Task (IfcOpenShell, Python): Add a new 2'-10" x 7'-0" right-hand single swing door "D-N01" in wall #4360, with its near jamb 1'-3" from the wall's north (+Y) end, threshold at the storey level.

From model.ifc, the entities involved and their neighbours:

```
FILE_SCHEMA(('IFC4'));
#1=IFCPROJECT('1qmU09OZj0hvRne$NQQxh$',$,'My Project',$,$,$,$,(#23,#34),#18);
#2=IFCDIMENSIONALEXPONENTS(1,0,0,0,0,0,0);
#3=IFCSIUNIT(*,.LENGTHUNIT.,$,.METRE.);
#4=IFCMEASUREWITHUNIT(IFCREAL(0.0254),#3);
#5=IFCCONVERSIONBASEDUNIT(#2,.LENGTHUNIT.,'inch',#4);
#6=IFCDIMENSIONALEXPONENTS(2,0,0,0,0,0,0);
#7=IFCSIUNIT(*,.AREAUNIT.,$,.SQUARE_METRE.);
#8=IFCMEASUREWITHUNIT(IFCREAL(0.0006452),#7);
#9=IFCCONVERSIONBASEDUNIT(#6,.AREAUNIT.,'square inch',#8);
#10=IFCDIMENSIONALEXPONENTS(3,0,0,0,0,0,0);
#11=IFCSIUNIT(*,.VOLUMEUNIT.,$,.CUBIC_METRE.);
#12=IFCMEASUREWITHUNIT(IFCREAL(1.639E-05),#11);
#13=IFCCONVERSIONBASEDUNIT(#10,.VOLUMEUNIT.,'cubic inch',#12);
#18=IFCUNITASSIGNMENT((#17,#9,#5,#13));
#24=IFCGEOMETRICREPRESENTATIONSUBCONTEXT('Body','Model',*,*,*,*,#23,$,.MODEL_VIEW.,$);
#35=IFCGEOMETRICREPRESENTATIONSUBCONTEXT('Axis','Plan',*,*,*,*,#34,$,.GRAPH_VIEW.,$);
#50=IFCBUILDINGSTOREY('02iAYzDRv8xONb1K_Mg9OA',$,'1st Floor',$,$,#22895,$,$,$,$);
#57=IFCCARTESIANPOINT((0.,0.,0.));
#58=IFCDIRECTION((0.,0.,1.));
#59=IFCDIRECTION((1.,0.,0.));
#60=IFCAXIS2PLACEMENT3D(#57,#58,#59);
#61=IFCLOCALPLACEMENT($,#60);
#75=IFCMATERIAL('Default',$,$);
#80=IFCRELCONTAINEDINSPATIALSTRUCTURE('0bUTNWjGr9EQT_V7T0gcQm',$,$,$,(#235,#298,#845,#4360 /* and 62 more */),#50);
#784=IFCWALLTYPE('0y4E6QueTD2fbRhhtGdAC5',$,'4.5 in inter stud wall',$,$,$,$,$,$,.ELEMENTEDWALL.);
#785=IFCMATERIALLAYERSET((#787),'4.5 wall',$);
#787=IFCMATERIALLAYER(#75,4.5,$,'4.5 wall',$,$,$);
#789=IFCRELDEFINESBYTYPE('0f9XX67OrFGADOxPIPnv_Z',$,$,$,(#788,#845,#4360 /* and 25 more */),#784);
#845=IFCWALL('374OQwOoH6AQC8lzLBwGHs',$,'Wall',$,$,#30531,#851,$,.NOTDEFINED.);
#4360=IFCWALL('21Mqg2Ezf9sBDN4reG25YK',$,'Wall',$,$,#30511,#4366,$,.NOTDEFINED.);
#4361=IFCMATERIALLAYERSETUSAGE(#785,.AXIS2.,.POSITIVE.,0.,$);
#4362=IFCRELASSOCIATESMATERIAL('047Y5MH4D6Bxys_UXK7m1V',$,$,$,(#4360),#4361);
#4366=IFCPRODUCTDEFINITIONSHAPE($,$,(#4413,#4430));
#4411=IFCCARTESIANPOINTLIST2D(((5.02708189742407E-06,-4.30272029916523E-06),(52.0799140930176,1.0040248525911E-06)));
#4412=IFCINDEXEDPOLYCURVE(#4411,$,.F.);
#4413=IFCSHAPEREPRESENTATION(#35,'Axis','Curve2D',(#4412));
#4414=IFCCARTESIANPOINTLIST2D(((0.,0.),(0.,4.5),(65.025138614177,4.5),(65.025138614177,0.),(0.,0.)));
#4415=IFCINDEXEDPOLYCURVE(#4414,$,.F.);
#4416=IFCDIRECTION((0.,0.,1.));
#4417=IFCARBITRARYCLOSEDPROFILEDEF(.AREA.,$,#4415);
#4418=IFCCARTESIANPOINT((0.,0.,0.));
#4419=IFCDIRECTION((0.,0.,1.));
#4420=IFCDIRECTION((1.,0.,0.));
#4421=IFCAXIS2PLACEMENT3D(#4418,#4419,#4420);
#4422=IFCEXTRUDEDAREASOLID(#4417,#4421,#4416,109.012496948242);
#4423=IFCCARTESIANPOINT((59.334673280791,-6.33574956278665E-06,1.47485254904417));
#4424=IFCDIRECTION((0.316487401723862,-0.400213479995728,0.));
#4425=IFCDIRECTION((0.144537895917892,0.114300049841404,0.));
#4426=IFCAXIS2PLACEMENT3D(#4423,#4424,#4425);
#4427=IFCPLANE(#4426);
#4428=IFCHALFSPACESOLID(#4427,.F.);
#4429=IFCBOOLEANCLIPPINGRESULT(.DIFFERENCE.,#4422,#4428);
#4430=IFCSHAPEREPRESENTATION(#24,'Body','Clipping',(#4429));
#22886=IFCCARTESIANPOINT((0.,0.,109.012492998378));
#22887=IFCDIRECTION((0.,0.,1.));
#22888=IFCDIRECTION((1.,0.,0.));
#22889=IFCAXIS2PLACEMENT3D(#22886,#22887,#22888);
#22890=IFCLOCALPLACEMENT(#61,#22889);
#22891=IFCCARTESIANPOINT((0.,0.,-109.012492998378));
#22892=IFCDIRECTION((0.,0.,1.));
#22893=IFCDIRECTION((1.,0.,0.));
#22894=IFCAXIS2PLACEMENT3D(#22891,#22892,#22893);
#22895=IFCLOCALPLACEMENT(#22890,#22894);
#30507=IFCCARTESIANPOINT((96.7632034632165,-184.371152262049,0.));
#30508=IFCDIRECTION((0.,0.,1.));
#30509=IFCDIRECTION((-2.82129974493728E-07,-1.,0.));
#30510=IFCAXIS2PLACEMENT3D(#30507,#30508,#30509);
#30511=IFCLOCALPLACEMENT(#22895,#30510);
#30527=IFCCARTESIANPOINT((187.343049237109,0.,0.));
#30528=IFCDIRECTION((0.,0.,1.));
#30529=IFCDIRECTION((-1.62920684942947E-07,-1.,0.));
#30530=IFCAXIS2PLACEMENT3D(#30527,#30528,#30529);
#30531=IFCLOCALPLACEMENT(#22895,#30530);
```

```python
import numpy as np
import ifcopenshell
import ifcopenshell.api.feature
import ifcopenshell.api.geometry
import ifcopenshell.api.root
import ifcopenshell.api.spatial
import ifcopenshell.geom
import ifcopenshell.util.element
import ifcopenshell.util.placement
import ifcopenshell.util.representation
import ifcopenshell.util.shape
import ifcopenshell.util.unit

model = ifcopenshell.open("model.ifc")
unit_scale = ifcopenshell.util.unit.calculate_unit_scale(model)
settings = ifcopenshell.geom.settings()


def volume(element):
    """Net volume in cubic metres, openings subtracted."""
    shape = ifcopenshell.geom.create_shape(settings, element)
    return ifcopenshell.util.shape.get_volume(shape.geometry)


wall = model.by_id(4360)
storey = ifcopenshell.util.element.get_container(wall, ifc_class="IfcBuildingStorey")
context = ifcopenshell.util.representation.get_context(model, "Model", "Body", "MODEL_VIEW")
before = volume(wall)

width, height, from_end, sill = 0.8636, 2.1336, 0.381, 0.0  # metres

# The wall runs along its own X axis, and the end named is its -X end.
wall_shape = ifcopenshell.geom.create_shape(settings, wall)
x, y, z = ifcopenshell.util.shape.get_vertices(wall_shape.geometry).T
start = x.min() + from_end
face, thickness = float(y.min()), float(y.max() - y.min())
wall_matrix = ifcopenshell.util.placement.get_local_placement(wall.ObjectPlacement)
level = ifcopenshell.util.placement.get_local_placement(storey.ObjectPlacement)[2, 3]


def in_wall(x, y):
    """Placement at x, y metres in the wall's axes, at sill height."""
    matrix = wall_matrix.copy()
    matrix[:, 3] = wall_matrix @ np.array([x / unit_scale, y / unit_scale, 0.0, 1.0])
    matrix[2, 3] = level + sill / unit_scale
    return matrix


# Opening: a box that overshoots both wall faces by 50 mm.
opening = ifcopenshell.api.root.create_entity(model, ifc_class="IfcOpeningElement", predefined_type="OPENING")
box = ifcopenshell.api.geometry.add_wall_representation(
    model, context=context, length=width, height=height, thickness=thickness + 0.1
)
ifcopenshell.api.geometry.assign_representation(model, product=opening, representation=box)
ifcopenshell.api.geometry.edit_object_placement(model, product=opening, matrix=in_wall(start, face - 0.05), is_si=False)
ifcopenshell.api.feature.add_feature(model, feature=opening, element=wall)

door = ifcopenshell.api.root.create_entity(model, ifc_class="IfcDoor", name="D-N01", predefined_type="DOOR")
door.OverallWidth, door.OverallHeight = width / unit_scale, height / unit_scale
door.OperationType = "SINGLE_SWING_RIGHT"
body = ifcopenshell.api.geometry.add_door_representation(
    model,
    context=context,
    overall_width=door.OverallWidth,
    overall_height=door.OverallHeight,
    operation_type="SINGLE_SWING_RIGHT",
    lining_properties={"LiningDepth": thickness / unit_scale, "ThresholdDepth": thickness / unit_scale},
)
ifcopenshell.api.geometry.assign_representation(model, product=door, representation=body)
ifcopenshell.api.spatial.assign_container(model, products=[door], relating_structure=storey)
ifcopenshell.api.feature.add_filling(model, opening=opening, element=door)

# The lining spans the wall, so the door starts at the wall face.
ifcopenshell.api.geometry.edit_object_placement(model, product=door, matrix=in_wall(start, face), is_si=False)

after = volume(wall)

print(f"wall volume {before:.3f} -> {after:.3f} m3")

model.write("model_rev.ifc")
```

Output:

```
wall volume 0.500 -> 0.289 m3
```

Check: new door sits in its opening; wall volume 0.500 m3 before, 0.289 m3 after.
